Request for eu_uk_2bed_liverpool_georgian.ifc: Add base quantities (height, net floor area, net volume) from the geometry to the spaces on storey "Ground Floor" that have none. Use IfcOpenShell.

First a look at what the model holds.

```python
import ifcopenshell
import ifcopenshell.util.element
import ifcopenshell.util.unit

model = ifcopenshell.open("eu_uk_2bed_liverpool_georgian.ifc")
print(model.schema)
for unit_type in ("LENGTHUNIT", "AREAUNIT", "VOLUMEUNIT"):
    print(unit_type, ifcopenshell.util.unit.calculate_unit_scale(model, unit_type))
storey = next(s for s in model.by_type("IfcBuildingStorey") if s.Name == "Ground Floor")
spaces = [e for e in ifcopenshell.util.element.get_decomposition(storey) if e.is_a("IfcSpace")]
for e in sorted(spaces, key=lambda e: e.id()):
    print(e.id(), e.is_a(), e.Name, list(ifcopenshell.util.element.get_psets(e, qtos_only=True)), sep=" | ")
```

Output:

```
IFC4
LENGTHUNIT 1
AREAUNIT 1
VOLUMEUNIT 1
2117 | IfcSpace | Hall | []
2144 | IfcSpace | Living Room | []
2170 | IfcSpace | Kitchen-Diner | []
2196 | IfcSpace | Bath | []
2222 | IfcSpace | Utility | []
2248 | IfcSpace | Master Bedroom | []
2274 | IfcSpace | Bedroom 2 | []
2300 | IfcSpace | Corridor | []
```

```python
import ifcopenshell
import ifcopenshell.api.pset
import ifcopenshell.geom
import ifcopenshell.util.element
import ifcopenshell.util.shape
import ifcopenshell.util.unit

model = ifcopenshell.open("eu_uk_2bed_liverpool_georgian.ifc")
unit_scale = ifcopenshell.util.unit.calculate_unit_scale(model)
area_scale = ifcopenshell.util.unit.calculate_unit_scale(model, "AREAUNIT")
volume_scale = ifcopenshell.util.unit.calculate_unit_scale(model, "VOLUMEUNIT")
settings = ifcopenshell.geom.settings()

storey = next(s for s in model.by_type("IfcBuildingStorey") if s.Name == "Ground Floor")
spaces = [e for e in ifcopenshell.util.element.get_decomposition(storey) if e.is_a("IfcSpace")]

for e in sorted(spaces, key=lambda e: e.id()):
    if ifcopenshell.util.element.get_psets(e, qtos_only=True, should_inherit=False):
        continue
    # Geometry comes back in metres, in the element's own axes.
    shape = ifcopenshell.geom.create_shape(settings, e)
    values = {
        "Height": ifcopenshell.util.shape.get_z(shape.geometry) / unit_scale,
        "NetFloorArea": ifcopenshell.util.shape.get_footprint_area(shape.geometry) / area_scale,
        "NetVolume": ifcopenshell.util.shape.get_volume(shape.geometry) / volume_scale,
    }
    qto = ifcopenshell.api.pset.add_qto(model, product=e, name="Qto_SpaceBaseQuantities")
    ifcopenshell.api.pset.edit_qto(model, qto=qto, properties=values)
    print(e.id(), {k: round(v, 3) for k, v in values.items()})

model.write("eu_uk_2bed_liverpool_georgian_edited.ifc")
```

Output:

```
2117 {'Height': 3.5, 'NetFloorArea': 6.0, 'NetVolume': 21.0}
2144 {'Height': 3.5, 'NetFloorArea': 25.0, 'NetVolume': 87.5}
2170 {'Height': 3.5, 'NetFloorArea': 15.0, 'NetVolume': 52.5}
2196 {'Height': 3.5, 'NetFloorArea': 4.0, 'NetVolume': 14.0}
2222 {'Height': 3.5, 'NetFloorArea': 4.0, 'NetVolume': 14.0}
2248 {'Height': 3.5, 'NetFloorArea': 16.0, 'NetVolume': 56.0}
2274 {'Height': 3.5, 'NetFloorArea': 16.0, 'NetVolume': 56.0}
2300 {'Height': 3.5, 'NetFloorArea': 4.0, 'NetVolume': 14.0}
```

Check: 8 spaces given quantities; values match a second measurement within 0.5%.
